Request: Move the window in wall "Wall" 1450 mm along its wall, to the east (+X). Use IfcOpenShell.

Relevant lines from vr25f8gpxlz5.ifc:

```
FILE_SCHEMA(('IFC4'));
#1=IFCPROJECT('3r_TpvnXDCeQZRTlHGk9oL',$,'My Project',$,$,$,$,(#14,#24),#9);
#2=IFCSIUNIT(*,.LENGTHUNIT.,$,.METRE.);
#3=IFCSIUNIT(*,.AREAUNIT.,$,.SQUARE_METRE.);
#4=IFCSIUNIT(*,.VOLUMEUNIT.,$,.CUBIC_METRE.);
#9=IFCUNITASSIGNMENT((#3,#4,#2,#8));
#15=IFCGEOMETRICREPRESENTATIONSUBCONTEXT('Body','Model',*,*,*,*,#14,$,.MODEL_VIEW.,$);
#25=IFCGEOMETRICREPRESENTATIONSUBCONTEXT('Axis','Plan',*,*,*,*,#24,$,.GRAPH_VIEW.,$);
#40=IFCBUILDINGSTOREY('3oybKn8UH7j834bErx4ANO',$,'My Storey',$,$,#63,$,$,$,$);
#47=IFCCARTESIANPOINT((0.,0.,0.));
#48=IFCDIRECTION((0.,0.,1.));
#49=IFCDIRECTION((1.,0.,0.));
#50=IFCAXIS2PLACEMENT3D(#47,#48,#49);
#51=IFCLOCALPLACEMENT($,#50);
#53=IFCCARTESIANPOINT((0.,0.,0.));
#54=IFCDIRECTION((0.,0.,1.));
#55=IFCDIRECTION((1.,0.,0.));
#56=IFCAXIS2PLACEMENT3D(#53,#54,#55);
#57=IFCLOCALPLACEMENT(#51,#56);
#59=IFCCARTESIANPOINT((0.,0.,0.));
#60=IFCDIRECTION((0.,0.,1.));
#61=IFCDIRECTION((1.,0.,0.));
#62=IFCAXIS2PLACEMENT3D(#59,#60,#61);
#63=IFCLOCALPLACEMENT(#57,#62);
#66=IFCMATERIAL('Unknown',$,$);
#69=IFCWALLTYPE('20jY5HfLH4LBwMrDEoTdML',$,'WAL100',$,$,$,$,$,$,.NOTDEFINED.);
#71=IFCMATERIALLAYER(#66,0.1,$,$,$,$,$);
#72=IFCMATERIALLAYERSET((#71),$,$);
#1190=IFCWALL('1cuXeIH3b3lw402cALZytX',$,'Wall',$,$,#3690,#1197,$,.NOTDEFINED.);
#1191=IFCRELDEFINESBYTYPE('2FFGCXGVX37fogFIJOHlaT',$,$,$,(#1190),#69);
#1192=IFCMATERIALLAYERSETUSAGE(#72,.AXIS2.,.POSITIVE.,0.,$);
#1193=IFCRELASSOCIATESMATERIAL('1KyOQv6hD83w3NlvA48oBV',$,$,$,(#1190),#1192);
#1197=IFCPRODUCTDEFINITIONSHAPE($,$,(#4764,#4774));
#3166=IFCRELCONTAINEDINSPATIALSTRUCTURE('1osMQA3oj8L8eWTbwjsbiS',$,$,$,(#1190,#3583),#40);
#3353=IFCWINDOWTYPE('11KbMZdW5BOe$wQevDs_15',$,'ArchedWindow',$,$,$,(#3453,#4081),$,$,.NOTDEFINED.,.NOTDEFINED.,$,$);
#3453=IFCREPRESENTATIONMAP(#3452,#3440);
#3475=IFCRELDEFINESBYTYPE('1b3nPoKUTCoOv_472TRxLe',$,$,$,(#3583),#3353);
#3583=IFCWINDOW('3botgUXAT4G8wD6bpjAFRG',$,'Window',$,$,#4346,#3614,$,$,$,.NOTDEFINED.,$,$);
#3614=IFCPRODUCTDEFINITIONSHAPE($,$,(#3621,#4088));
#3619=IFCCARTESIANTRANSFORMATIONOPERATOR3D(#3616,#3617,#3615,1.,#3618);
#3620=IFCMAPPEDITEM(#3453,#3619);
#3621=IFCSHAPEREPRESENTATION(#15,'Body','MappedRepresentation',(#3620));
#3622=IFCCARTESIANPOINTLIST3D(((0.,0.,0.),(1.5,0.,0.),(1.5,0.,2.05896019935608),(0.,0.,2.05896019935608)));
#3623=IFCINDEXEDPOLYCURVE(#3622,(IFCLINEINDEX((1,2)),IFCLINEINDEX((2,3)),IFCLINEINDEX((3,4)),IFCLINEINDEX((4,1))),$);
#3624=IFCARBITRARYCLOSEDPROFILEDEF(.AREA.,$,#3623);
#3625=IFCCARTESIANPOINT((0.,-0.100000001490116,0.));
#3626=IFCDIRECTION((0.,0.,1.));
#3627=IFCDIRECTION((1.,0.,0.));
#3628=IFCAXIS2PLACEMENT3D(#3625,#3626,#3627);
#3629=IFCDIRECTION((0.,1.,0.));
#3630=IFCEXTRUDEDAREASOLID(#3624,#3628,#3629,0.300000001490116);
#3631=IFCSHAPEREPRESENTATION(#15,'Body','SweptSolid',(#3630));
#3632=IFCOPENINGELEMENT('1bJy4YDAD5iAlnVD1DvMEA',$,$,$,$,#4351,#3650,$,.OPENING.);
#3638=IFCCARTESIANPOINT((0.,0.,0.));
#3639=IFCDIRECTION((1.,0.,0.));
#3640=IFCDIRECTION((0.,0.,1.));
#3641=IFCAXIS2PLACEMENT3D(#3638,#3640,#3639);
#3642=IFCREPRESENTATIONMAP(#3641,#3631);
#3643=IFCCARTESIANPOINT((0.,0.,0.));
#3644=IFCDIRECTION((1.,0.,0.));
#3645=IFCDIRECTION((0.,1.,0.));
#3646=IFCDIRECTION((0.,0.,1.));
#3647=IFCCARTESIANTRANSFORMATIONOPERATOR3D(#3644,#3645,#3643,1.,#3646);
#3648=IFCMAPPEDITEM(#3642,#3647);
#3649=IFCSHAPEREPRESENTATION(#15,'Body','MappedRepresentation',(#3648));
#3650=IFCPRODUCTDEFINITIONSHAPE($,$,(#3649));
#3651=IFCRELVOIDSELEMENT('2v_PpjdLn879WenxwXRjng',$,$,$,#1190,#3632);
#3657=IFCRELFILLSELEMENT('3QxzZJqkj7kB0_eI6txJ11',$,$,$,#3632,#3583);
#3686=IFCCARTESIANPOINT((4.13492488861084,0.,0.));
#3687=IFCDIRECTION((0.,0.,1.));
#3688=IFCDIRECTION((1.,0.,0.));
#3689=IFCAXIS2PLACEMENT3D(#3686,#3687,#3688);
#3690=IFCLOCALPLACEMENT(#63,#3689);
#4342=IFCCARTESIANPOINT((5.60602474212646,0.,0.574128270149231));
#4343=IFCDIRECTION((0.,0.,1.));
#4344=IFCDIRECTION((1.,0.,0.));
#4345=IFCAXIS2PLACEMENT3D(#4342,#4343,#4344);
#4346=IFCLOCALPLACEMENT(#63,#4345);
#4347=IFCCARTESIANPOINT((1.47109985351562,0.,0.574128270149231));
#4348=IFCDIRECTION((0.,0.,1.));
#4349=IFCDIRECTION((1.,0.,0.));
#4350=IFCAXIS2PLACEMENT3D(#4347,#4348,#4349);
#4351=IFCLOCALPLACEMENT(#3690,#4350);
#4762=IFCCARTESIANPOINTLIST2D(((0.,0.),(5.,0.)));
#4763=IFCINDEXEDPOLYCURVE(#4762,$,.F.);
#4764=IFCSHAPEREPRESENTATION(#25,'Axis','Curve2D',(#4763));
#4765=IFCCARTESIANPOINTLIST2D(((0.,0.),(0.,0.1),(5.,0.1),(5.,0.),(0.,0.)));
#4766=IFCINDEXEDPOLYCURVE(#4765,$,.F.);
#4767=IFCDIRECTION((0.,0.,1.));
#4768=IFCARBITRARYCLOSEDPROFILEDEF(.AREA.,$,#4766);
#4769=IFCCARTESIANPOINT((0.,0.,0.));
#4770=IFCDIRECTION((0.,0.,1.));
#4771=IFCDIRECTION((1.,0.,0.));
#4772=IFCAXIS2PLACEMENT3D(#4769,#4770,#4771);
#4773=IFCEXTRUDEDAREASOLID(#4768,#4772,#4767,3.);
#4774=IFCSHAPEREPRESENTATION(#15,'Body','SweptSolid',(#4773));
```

```python
import ifcopenshell
import ifcopenshell.api.geometry
import ifcopenshell.util.placement

model = ifcopenshell.open("vr25f8gpxlz5.ifc")

window = model.by_guid("3botgUXAT4G8wD6bpjAFRG")
opening = window.FillsVoids[0].RelatingOpeningElement
wall = opening.VoidsElements[0].RelatingBuildingElement

wall_matrix = ifcopenshell.util.placement.get_local_placement(wall.ObjectPlacement)
shift = wall_matrix[:3, 0] * 1.45
before = ifcopenshell.util.placement.get_local_placement(window.ObjectPlacement)[:3, 3].copy()

# The window is not placed relative to its opening, so move both.
for product in (opening, window):
    matrix = ifcopenshell.util.placement.get_local_placement(product.ObjectPlacement)
    matrix[:3, 3] += shift
    ifcopenshell.api.geometry.edit_object_placement(model, product=product, matrix=matrix, is_si=False)

after = ifcopenshell.util.placement.get_local_placement(window.ObjectPlacement)[:3, 3]
print("window moved by", (after - before).round(3) + 0.0)

model.write("vr25f8gpxlz5_v2.ifc")
```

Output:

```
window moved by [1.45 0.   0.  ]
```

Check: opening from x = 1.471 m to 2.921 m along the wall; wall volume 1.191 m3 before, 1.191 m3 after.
